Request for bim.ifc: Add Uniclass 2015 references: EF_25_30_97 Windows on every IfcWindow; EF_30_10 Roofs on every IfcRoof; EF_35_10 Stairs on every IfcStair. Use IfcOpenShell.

First a look at what the model holds.

```python
import ifcopenshell

model = ifcopenshell.open("bim.ifc")
print(model.schema)
print("classifications:", [c.Name for c in model.by_type("IfcClassification")])
for ifc_class in ("IfcDoor", "IfcRoof", "IfcStair", "IfcWall", "IfcWindow"):
    print(ifc_class, len(model.by_type(ifc_class)))
```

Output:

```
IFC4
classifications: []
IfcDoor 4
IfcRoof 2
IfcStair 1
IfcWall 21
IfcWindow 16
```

```python
import ifcopenshell
import ifcopenshell.api.classification

model = ifcopenshell.open("bim.ifc")

system = ifcopenshell.api.classification.add_classification(model, classification="Uniclass 2015")

codes = {
    "IfcWindow": ("EF_25_30_97", "Windows"),
    "IfcRoof": ("EF_30_10", "Roofs"),
    "IfcStair": ("EF_35_10", "Stairs"),
}
for ifc_class, (code, name) in codes.items():
    products = model.by_type(ifc_class)
    ifcopenshell.api.classification.add_reference(
        model, products=products, classification=system, identification=code, name=name
    )
    print(code, len(products))

model.write("bim_edited.ifc")
```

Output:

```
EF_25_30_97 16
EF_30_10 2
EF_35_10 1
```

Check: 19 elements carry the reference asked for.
